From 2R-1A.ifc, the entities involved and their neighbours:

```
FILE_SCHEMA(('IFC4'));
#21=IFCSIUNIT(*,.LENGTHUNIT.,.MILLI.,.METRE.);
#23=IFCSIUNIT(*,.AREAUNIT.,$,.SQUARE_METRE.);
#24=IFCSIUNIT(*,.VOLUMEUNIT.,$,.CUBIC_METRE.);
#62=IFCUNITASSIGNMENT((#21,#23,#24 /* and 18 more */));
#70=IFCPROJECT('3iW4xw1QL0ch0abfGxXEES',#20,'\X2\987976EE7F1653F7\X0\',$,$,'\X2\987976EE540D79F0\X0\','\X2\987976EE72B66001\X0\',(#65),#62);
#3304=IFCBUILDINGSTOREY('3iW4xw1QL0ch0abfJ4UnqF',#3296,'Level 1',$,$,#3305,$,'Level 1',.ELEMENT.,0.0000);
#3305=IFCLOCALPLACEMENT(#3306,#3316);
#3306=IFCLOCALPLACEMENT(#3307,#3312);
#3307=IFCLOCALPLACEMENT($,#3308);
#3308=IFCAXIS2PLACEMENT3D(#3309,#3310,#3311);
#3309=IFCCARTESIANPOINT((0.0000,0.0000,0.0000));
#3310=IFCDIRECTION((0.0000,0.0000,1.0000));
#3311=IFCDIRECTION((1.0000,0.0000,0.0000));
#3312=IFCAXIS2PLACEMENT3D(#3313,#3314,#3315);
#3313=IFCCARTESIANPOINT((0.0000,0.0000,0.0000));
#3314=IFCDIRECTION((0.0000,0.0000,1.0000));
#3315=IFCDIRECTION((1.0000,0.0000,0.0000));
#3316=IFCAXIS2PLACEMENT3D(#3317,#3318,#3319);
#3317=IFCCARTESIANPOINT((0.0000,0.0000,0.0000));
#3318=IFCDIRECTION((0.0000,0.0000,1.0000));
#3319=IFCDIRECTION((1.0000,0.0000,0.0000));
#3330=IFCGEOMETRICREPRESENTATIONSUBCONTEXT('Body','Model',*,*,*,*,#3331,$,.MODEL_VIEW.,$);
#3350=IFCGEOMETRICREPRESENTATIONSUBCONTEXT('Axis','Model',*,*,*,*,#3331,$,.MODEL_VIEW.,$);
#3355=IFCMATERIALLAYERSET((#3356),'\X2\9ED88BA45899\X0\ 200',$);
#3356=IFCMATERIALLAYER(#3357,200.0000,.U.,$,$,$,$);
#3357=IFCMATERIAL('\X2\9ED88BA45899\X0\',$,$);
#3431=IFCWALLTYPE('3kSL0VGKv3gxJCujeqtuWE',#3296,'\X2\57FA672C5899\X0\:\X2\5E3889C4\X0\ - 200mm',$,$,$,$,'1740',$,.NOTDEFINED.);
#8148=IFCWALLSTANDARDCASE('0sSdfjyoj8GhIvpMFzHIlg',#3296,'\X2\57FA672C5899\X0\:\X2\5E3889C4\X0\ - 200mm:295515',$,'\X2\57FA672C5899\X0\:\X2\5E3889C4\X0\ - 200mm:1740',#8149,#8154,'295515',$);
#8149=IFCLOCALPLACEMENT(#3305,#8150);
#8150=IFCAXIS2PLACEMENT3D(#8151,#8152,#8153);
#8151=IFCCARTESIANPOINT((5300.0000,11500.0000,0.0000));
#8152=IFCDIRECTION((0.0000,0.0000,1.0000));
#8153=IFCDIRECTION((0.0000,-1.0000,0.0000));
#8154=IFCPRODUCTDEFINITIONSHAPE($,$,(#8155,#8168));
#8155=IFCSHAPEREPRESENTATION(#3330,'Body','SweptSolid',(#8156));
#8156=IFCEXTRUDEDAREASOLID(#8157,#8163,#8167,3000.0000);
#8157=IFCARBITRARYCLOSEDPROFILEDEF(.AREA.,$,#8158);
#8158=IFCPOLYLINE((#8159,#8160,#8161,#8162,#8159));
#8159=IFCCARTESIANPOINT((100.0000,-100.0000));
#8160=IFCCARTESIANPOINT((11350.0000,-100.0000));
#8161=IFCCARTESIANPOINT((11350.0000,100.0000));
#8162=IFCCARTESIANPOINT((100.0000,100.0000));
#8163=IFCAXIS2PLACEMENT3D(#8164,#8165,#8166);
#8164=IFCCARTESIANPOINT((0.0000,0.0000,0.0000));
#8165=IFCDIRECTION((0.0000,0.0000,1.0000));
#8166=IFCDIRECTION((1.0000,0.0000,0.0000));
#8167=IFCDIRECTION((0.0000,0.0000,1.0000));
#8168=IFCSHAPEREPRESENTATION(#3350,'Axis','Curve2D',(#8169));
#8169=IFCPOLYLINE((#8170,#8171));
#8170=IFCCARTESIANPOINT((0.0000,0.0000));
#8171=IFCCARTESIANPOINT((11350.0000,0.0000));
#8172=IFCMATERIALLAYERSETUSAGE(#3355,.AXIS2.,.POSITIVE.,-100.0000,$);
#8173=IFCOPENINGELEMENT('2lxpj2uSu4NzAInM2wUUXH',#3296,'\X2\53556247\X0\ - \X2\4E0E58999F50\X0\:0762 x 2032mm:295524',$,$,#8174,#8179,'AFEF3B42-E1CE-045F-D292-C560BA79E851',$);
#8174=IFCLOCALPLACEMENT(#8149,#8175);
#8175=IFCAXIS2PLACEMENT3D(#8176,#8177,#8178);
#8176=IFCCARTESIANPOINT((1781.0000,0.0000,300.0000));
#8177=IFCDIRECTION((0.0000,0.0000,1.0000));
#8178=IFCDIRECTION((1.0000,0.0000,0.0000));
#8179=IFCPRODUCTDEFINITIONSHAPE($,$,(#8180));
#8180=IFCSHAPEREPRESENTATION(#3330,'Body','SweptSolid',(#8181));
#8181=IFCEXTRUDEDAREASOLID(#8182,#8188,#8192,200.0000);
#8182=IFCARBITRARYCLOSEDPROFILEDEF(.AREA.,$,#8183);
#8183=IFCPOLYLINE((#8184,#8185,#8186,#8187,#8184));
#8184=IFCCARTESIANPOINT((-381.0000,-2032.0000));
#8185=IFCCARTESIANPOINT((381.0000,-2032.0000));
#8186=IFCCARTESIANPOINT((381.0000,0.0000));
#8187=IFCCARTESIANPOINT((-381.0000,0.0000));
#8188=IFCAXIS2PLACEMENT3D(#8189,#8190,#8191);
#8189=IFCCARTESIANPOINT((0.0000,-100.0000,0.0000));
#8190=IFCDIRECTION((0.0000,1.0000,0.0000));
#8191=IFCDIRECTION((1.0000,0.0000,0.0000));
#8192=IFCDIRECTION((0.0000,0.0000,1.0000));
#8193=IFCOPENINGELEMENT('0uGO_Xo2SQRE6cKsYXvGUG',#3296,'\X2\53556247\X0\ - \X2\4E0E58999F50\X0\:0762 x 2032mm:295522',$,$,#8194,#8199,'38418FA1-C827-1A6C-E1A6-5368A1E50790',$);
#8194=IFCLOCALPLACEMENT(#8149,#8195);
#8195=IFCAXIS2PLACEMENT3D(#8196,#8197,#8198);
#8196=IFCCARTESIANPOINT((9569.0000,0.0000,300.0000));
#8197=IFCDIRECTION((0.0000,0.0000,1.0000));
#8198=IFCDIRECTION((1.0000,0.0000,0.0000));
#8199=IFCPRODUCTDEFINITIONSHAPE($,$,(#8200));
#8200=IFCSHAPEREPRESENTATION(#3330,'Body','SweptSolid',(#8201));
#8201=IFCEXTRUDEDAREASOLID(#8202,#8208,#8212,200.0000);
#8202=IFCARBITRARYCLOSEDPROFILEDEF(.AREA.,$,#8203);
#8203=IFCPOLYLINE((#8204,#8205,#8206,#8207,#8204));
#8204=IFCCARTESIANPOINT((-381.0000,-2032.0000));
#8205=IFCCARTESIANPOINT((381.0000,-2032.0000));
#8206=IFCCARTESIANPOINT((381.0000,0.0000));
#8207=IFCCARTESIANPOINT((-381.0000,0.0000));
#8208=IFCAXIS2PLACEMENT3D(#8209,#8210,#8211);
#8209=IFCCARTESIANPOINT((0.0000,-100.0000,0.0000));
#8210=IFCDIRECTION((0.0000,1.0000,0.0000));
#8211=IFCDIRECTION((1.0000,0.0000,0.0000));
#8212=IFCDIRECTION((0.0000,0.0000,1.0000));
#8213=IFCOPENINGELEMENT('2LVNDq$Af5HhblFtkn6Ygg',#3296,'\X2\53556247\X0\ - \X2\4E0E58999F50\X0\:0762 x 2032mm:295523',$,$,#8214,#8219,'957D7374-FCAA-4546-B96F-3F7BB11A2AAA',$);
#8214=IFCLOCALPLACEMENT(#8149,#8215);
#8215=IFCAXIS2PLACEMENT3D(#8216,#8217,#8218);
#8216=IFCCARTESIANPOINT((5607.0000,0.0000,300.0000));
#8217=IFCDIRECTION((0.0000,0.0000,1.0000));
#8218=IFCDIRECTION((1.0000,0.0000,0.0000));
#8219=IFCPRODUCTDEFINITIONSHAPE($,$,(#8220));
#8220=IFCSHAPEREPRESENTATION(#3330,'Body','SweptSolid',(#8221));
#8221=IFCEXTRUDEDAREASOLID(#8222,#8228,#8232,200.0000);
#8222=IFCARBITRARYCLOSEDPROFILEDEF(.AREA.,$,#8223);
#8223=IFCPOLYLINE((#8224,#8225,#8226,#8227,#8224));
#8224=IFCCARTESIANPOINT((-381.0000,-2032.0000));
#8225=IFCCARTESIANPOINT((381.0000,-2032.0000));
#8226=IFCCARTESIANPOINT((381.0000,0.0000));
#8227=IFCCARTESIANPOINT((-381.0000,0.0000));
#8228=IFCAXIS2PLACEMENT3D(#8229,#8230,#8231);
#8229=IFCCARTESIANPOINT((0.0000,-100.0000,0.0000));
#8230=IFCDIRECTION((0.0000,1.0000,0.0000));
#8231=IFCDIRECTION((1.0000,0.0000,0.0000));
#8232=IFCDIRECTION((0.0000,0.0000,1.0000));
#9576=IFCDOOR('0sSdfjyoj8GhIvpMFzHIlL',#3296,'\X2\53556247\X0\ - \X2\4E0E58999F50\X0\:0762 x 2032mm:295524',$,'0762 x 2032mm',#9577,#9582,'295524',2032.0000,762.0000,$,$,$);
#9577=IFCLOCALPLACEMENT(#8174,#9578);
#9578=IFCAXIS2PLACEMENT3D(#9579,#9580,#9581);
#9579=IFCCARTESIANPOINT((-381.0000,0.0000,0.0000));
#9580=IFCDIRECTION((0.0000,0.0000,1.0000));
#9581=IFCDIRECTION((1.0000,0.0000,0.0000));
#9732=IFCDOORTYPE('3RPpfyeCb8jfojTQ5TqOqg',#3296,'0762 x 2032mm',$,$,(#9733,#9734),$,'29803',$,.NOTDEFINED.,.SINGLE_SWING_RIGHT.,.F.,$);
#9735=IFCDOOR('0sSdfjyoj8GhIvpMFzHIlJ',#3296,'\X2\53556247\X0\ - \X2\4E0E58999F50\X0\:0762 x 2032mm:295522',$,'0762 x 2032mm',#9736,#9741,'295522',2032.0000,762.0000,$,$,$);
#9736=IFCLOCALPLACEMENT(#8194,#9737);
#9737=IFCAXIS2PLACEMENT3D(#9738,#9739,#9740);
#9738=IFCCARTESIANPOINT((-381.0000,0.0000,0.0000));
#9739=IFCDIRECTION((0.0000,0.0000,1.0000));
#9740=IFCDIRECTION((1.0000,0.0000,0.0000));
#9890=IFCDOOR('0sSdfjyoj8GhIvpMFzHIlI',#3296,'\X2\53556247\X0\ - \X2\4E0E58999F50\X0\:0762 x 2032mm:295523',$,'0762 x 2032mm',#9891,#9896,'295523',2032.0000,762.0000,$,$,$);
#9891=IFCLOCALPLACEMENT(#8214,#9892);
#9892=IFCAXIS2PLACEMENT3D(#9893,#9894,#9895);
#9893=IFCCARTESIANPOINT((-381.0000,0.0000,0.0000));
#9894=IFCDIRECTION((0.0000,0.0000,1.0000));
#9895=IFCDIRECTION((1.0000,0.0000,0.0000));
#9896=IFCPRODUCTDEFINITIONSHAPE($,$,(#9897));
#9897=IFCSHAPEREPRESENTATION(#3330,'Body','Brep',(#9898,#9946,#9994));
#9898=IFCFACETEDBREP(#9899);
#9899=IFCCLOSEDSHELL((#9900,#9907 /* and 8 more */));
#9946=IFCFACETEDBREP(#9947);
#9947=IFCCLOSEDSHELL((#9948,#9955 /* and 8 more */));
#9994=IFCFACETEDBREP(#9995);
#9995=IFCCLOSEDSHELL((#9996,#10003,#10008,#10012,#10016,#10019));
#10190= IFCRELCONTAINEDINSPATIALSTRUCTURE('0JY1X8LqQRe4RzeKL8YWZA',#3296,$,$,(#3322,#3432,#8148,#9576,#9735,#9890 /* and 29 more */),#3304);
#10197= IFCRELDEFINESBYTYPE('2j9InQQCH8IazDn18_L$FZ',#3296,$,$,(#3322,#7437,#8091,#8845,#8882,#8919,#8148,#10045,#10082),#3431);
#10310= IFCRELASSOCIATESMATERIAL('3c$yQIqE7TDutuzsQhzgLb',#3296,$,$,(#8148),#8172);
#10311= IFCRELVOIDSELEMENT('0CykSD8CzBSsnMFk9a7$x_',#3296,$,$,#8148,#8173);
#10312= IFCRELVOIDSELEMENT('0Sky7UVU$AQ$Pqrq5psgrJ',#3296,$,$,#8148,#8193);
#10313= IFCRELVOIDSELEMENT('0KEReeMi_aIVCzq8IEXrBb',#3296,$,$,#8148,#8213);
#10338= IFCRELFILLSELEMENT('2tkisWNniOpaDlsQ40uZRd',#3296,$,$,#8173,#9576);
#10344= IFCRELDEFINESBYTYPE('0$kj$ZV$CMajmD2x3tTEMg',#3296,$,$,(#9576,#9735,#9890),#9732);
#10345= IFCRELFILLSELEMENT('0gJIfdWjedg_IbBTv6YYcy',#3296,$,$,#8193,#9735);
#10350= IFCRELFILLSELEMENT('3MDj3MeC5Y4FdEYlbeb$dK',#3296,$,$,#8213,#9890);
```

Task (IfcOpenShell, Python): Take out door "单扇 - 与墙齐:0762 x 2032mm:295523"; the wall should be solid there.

```python
import ifcopenshell
import ifcopenshell.api.feature
import ifcopenshell.api.root
import ifcopenshell.geom
import ifcopenshell.util.shape

model = ifcopenshell.open("2R-1A.ifc")
settings = ifcopenshell.geom.settings()


def volume(element):
    """Net volume in cubic metres, openings subtracted."""
    shape = ifcopenshell.geom.create_shape(settings, element)
    return ifcopenshell.util.shape.get_volume(shape.geometry)


door = model.by_guid("0sSdfjyoj8GhIvpMFzHIlI")
opening = door.FillsVoids[0].RelatingOpeningElement
wall = opening.VoidsElements[0].RelatingBuildingElement
before = volume(wall)

ifcopenshell.api.root.remove_product(model, product=door)
ifcopenshell.api.feature.remove_feature(model, feature=opening)

after = volume(wall)

print(f"wall volume {before:.3f} -> {after:.3f} m3")

model.write("2R-1A_rev.ifc")
```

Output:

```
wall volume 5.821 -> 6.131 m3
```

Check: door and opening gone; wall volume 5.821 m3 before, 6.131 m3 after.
